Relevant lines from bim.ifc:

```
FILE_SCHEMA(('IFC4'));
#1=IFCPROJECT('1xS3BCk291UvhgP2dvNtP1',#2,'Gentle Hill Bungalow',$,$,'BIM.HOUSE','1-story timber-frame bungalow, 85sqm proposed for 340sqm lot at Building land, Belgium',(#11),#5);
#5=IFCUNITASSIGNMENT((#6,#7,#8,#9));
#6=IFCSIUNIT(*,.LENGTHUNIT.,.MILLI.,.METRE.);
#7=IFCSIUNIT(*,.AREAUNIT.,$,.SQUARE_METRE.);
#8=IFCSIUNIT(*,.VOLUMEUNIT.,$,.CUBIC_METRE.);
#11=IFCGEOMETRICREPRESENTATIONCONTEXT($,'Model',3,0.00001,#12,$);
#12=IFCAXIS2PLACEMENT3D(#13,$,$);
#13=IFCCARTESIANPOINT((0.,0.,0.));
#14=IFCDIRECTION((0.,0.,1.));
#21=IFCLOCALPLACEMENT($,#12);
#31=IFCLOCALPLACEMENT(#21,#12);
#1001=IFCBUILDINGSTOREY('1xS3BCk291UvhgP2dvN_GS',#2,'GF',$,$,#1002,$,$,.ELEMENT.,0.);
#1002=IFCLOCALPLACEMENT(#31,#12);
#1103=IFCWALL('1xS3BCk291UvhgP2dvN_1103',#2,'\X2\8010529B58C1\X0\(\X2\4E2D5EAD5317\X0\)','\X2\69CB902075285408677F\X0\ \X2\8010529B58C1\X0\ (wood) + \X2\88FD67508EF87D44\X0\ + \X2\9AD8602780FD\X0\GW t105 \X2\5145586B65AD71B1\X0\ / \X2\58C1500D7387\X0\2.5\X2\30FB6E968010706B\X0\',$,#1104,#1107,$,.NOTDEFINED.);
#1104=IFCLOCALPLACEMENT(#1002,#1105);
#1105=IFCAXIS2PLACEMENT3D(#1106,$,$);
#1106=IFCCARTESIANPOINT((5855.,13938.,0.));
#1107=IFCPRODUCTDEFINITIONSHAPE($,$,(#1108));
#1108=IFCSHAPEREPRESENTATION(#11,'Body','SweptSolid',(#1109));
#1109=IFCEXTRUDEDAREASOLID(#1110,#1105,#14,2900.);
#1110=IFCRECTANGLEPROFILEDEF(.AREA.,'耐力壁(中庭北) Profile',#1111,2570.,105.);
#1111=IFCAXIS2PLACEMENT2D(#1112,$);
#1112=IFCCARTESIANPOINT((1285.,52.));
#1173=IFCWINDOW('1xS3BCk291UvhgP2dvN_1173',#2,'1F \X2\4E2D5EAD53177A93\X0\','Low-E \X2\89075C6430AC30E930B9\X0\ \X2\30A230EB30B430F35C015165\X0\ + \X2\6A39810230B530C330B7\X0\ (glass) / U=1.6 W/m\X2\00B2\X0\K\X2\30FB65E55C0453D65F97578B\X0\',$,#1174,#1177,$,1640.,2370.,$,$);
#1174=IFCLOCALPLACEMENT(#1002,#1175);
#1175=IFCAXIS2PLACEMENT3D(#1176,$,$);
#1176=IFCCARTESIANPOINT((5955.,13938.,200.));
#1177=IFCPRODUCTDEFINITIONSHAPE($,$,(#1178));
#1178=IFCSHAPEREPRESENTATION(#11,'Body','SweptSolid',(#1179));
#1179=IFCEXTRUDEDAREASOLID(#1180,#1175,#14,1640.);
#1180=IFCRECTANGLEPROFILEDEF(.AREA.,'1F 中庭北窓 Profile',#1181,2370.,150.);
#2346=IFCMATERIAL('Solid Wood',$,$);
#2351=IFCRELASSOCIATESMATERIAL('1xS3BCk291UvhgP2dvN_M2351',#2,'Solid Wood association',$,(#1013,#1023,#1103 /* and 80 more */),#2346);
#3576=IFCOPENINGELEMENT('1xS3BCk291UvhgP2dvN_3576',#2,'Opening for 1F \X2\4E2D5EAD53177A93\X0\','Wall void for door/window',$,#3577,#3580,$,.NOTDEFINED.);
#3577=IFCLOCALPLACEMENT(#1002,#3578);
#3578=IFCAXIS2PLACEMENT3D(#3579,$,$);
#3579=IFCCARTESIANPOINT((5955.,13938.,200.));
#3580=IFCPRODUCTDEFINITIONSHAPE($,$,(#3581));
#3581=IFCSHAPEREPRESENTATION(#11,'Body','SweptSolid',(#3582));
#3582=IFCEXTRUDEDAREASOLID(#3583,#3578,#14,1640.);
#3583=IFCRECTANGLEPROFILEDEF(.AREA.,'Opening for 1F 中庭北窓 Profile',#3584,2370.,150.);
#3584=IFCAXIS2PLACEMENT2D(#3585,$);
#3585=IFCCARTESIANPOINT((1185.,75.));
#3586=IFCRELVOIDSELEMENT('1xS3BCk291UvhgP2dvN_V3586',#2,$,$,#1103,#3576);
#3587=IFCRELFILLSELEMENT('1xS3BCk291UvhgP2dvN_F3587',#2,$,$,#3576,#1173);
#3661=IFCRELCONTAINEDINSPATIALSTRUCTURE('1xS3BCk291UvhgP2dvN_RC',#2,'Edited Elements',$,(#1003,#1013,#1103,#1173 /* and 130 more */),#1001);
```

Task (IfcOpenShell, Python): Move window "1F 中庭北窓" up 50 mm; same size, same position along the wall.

```python
import numpy as np
import ifcopenshell
import ifcopenshell.api.geometry
import ifcopenshell.util.placement
import ifcopenshell.util.unit

model = ifcopenshell.open("bim.ifc")
unit_scale = ifcopenshell.util.unit.calculate_unit_scale(model)

window = model.by_id(1173)
opening = window.FillsVoids[0].RelatingOpeningElement
dz = 0.05 / unit_scale

shift = np.array([0.0, 0.0, dz])
# The window is not placed relative to its opening, so move both.
for product in (opening, window):
    matrix = ifcopenshell.util.placement.get_local_placement(product.ObjectPlacement)
    matrix[:3, 3] += shift
    ifcopenshell.api.geometry.edit_object_placement(model, product=product, matrix=matrix, is_si=False)

print(f"moved by {dz * unit_scale:+.3f} m")

model.write("bim-out.ifc")
```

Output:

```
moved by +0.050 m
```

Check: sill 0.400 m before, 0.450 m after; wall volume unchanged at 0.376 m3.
